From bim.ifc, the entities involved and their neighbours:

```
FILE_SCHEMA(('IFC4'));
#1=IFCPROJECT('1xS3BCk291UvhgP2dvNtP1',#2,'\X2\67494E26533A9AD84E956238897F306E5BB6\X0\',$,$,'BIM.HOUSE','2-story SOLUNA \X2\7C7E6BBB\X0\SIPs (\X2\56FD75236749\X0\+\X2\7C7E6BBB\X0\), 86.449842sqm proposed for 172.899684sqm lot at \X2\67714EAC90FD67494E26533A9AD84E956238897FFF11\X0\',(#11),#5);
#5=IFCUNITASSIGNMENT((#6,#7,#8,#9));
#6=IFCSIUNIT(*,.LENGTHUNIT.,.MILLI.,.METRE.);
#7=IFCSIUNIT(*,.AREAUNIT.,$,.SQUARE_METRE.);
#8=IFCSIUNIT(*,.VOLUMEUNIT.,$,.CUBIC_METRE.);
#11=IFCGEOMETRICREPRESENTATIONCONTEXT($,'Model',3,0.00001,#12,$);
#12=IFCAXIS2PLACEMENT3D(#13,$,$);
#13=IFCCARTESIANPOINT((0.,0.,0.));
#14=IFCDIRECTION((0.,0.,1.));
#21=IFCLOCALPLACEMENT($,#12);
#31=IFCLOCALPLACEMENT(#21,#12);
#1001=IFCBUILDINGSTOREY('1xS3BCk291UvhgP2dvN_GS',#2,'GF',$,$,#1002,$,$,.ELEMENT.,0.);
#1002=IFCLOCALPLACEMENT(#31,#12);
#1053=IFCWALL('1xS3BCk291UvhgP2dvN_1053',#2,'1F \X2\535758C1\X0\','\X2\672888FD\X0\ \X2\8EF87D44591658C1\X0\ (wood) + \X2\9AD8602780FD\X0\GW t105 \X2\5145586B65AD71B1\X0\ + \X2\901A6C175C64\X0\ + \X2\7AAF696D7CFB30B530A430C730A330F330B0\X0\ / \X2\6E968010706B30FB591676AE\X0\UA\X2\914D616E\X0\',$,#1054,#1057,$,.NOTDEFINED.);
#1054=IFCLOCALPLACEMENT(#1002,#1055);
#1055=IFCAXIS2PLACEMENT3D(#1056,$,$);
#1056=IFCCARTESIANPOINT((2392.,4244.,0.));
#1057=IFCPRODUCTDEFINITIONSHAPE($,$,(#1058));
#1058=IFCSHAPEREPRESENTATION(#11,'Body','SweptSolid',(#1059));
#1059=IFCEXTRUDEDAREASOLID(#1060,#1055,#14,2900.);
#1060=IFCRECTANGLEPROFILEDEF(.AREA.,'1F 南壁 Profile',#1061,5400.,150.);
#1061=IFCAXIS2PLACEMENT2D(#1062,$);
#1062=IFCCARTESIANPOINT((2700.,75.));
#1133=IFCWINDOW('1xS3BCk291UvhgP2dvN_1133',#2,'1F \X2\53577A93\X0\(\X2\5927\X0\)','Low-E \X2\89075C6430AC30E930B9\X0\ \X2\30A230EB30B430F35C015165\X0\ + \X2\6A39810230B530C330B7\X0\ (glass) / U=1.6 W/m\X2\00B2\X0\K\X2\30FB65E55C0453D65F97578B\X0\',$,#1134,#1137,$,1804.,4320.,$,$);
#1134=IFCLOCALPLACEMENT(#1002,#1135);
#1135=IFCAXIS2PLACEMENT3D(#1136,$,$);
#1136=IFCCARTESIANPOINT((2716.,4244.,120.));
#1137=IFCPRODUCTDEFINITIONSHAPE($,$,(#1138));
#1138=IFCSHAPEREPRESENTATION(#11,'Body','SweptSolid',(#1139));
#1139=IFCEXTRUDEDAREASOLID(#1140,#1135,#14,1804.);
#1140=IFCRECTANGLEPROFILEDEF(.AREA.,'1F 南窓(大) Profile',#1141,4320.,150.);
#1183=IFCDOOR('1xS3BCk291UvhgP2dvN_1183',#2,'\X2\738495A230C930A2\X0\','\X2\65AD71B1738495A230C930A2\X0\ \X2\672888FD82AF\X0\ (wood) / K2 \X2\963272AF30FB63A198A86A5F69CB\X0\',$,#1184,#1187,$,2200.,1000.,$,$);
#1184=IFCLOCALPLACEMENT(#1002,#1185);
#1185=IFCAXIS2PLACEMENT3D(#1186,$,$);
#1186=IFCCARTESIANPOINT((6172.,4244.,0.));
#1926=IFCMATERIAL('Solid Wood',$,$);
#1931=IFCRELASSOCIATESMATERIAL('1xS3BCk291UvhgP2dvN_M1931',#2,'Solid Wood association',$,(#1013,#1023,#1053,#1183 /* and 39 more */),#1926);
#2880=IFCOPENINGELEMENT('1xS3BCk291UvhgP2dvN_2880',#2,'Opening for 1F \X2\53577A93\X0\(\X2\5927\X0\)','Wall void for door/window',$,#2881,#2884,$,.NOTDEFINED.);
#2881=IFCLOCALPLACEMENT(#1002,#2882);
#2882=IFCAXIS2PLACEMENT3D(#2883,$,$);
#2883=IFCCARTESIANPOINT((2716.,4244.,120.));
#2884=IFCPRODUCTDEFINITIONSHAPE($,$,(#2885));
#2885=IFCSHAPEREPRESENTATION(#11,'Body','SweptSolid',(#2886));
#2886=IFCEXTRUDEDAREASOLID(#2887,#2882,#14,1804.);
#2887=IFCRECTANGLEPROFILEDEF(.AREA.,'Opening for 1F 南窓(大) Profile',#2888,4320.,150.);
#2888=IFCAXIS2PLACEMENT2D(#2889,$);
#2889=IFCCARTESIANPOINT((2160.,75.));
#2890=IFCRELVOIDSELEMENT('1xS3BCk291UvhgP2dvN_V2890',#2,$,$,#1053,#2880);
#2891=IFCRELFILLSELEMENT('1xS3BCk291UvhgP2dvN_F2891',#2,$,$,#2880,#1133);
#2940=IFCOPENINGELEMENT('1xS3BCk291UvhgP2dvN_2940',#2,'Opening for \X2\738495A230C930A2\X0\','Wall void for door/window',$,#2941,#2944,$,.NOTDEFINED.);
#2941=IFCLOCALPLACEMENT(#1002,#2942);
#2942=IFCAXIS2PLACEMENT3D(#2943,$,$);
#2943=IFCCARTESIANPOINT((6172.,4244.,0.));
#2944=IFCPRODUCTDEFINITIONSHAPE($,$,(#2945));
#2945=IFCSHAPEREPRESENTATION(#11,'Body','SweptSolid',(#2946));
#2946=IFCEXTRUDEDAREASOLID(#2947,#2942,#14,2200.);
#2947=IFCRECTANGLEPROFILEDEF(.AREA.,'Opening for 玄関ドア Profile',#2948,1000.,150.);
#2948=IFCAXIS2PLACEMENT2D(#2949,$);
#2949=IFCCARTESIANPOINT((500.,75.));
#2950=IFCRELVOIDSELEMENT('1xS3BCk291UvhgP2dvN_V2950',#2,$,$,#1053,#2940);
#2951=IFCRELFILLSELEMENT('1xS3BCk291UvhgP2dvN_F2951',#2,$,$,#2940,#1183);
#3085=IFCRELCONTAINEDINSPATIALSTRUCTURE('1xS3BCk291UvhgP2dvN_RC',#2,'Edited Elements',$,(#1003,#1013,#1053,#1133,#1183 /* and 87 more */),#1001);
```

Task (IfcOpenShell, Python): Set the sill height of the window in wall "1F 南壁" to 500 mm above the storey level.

```python
import numpy as np
import ifcopenshell
import ifcopenshell.api.geometry
import ifcopenshell.geom
import ifcopenshell.util.element
import ifcopenshell.util.placement
import ifcopenshell.util.shape
import ifcopenshell.util.unit

model = ifcopenshell.open("bim.ifc")
unit_scale = ifcopenshell.util.unit.calculate_unit_scale(model)

window = model.by_id(1133)
opening = window.FillsVoids[0].RelatingOpeningElement
storey = ifcopenshell.util.element.get_container(window, ifc_class="IfcBuildingStorey")
level = ifcopenshell.util.placement.get_local_placement(storey.ObjectPlacement)[2, 3]

# The opening's origin need not be at the sill, so measure its lowest point.
shape = ifcopenshell.geom.create_shape(ifcopenshell.geom.settings(), opening)
bottom = ifcopenshell.util.shape.get_shape_bottom_elevation(shape, shape.geometry) / unit_scale
dz = level + 500.0 - bottom

shift = np.array([0.0, 0.0, dz])
# The window is not placed relative to its opening, so move both.
for product in (opening, window):
    matrix = ifcopenshell.util.placement.get_local_placement(product.ObjectPlacement)
    matrix[:3, 3] += shift
    ifcopenshell.api.geometry.edit_object_placement(model, product=product, matrix=matrix, is_si=False)

print(f"moved by {dz * unit_scale:+.3f} m")

model.write("bim_rev.ifc")
```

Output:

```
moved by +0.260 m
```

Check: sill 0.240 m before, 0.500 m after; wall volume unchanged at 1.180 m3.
